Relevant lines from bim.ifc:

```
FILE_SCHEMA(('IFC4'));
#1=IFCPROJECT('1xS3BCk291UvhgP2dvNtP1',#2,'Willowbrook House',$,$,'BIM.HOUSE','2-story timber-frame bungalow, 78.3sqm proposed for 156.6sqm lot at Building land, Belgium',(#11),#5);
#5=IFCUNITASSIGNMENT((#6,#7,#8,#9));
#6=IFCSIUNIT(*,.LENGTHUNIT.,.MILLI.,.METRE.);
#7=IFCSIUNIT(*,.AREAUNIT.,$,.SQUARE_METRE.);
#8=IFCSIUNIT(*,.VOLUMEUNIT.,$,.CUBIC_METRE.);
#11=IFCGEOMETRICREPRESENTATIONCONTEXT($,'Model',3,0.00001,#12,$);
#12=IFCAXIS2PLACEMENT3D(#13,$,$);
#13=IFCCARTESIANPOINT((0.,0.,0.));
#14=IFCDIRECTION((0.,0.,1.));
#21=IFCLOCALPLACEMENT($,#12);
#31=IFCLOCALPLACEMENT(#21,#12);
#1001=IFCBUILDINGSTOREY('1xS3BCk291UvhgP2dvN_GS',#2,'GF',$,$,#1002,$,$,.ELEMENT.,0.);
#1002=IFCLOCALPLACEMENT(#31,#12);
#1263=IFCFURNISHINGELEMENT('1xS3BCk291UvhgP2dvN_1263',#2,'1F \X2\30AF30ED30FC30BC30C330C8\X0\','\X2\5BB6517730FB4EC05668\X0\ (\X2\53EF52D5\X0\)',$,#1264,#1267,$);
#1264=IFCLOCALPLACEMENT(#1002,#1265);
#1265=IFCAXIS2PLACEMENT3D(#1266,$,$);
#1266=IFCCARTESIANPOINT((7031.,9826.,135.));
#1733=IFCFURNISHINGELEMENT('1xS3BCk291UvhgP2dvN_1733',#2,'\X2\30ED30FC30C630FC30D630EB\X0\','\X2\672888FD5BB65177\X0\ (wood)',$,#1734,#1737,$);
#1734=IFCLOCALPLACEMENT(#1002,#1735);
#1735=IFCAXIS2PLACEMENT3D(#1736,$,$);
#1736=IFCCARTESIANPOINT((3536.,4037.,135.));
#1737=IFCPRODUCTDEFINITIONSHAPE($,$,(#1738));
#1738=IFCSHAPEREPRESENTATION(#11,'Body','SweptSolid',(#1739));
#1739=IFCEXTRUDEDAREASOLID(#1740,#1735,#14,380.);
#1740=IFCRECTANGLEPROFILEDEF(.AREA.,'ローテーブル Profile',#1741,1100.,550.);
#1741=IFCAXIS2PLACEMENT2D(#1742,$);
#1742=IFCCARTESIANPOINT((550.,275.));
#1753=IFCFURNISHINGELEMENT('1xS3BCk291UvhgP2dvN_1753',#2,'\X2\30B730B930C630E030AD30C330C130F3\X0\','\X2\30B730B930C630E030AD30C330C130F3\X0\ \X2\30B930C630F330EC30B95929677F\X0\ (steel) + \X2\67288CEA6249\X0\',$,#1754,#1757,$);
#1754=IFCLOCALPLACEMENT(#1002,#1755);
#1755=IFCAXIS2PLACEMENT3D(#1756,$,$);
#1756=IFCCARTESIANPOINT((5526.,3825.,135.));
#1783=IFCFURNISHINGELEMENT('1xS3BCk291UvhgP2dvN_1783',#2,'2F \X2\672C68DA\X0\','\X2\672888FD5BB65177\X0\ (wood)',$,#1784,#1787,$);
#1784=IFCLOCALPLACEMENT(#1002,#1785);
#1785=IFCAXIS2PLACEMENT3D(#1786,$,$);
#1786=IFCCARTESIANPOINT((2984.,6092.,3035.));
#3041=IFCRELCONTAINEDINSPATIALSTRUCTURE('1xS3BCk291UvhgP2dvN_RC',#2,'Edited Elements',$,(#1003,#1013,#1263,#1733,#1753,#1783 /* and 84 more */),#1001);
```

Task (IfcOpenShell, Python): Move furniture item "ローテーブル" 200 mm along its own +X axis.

```python
import ifcopenshell
import ifcopenshell.api.geometry
import ifcopenshell.util.placement
import ifcopenshell.util.unit

model = ifcopenshell.open("bim.ifc")
unit_scale = ifcopenshell.util.unit.calculate_unit_scale(model)

item = model.by_id(1733)
matrix = ifcopenshell.util.placement.get_local_placement(item.ObjectPlacement)
matrix[:3, 3] += matrix[:3, 0] * 0.2 / unit_scale
ifcopenshell.api.geometry.edit_object_placement(model, product=item, matrix=matrix, is_si=False)

print(ifcopenshell.util.placement.get_local_placement(item.ObjectPlacement).round(3) + 0.0)

model.write("bim_updated.ifc")
```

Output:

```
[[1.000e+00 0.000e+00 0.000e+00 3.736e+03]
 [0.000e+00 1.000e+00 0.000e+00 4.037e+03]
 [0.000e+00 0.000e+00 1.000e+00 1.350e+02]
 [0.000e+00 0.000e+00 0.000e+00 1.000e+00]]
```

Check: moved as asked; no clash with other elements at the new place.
